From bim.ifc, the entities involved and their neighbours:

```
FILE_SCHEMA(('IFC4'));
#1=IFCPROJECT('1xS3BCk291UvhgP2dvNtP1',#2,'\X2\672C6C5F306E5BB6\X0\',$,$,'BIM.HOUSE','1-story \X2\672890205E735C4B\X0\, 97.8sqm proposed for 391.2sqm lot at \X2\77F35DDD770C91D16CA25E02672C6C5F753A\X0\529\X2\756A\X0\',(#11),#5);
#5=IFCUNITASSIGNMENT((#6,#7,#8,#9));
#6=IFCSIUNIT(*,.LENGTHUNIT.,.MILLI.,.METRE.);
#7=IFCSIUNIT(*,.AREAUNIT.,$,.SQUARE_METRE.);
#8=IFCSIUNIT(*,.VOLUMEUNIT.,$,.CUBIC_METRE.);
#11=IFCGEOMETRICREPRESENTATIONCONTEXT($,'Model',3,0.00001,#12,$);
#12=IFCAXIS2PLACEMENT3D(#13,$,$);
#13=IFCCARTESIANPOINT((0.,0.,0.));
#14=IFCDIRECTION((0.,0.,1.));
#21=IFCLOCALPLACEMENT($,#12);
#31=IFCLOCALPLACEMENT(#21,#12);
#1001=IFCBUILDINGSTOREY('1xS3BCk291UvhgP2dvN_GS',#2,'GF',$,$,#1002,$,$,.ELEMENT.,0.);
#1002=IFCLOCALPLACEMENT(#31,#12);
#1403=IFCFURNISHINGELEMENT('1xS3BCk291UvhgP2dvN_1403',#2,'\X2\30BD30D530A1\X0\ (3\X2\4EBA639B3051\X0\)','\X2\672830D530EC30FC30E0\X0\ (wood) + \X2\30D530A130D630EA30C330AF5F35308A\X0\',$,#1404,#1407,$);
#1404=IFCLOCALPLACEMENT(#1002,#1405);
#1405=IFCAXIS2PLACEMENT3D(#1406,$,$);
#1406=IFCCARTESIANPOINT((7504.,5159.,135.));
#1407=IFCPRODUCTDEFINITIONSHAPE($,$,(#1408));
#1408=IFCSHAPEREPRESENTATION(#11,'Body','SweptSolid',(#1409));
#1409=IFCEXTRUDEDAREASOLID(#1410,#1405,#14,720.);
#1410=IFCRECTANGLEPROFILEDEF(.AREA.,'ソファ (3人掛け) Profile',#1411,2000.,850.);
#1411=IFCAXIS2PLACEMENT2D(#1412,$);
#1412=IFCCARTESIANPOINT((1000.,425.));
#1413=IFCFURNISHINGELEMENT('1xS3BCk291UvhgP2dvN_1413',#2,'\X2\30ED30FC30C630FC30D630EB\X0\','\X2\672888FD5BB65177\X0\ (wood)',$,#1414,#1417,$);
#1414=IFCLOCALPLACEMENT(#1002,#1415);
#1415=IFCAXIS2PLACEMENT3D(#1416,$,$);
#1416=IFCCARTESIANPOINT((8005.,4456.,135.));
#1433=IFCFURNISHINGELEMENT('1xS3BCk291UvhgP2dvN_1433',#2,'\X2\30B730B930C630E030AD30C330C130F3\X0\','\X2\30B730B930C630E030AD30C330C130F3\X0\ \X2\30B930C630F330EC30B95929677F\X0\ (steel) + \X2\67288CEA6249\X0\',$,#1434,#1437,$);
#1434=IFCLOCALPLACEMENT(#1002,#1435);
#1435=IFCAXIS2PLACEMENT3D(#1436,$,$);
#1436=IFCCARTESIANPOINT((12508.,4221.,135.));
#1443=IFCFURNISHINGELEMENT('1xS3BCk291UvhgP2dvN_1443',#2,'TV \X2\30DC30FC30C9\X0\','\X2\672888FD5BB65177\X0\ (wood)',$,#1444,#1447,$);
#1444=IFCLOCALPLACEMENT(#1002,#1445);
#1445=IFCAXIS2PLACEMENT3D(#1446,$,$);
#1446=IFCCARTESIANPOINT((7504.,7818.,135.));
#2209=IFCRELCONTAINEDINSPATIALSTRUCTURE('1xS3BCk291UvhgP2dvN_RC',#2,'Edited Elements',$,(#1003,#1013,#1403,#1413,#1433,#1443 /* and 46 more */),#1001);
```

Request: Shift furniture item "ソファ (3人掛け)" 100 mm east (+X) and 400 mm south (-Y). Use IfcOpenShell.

```python
import ifcopenshell
import ifcopenshell.api.geometry
import ifcopenshell.util.placement

model = ifcopenshell.open("bim.ifc")

item = model.by_id(1403)
matrix = ifcopenshell.util.placement.get_local_placement(item.ObjectPlacement)
matrix[0, 3] += 100.0
matrix[1, 3] -= 400.0
ifcopenshell.api.geometry.edit_object_placement(model, product=item, matrix=matrix, is_si=False)

print(ifcopenshell.util.placement.get_local_placement(item.ObjectPlacement).round(3) + 0.0)

model.write("bim_rev.ifc")
```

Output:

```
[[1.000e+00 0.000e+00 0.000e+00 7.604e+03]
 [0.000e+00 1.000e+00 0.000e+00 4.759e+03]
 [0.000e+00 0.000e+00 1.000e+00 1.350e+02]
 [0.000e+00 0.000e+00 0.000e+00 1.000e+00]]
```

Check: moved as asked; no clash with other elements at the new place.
